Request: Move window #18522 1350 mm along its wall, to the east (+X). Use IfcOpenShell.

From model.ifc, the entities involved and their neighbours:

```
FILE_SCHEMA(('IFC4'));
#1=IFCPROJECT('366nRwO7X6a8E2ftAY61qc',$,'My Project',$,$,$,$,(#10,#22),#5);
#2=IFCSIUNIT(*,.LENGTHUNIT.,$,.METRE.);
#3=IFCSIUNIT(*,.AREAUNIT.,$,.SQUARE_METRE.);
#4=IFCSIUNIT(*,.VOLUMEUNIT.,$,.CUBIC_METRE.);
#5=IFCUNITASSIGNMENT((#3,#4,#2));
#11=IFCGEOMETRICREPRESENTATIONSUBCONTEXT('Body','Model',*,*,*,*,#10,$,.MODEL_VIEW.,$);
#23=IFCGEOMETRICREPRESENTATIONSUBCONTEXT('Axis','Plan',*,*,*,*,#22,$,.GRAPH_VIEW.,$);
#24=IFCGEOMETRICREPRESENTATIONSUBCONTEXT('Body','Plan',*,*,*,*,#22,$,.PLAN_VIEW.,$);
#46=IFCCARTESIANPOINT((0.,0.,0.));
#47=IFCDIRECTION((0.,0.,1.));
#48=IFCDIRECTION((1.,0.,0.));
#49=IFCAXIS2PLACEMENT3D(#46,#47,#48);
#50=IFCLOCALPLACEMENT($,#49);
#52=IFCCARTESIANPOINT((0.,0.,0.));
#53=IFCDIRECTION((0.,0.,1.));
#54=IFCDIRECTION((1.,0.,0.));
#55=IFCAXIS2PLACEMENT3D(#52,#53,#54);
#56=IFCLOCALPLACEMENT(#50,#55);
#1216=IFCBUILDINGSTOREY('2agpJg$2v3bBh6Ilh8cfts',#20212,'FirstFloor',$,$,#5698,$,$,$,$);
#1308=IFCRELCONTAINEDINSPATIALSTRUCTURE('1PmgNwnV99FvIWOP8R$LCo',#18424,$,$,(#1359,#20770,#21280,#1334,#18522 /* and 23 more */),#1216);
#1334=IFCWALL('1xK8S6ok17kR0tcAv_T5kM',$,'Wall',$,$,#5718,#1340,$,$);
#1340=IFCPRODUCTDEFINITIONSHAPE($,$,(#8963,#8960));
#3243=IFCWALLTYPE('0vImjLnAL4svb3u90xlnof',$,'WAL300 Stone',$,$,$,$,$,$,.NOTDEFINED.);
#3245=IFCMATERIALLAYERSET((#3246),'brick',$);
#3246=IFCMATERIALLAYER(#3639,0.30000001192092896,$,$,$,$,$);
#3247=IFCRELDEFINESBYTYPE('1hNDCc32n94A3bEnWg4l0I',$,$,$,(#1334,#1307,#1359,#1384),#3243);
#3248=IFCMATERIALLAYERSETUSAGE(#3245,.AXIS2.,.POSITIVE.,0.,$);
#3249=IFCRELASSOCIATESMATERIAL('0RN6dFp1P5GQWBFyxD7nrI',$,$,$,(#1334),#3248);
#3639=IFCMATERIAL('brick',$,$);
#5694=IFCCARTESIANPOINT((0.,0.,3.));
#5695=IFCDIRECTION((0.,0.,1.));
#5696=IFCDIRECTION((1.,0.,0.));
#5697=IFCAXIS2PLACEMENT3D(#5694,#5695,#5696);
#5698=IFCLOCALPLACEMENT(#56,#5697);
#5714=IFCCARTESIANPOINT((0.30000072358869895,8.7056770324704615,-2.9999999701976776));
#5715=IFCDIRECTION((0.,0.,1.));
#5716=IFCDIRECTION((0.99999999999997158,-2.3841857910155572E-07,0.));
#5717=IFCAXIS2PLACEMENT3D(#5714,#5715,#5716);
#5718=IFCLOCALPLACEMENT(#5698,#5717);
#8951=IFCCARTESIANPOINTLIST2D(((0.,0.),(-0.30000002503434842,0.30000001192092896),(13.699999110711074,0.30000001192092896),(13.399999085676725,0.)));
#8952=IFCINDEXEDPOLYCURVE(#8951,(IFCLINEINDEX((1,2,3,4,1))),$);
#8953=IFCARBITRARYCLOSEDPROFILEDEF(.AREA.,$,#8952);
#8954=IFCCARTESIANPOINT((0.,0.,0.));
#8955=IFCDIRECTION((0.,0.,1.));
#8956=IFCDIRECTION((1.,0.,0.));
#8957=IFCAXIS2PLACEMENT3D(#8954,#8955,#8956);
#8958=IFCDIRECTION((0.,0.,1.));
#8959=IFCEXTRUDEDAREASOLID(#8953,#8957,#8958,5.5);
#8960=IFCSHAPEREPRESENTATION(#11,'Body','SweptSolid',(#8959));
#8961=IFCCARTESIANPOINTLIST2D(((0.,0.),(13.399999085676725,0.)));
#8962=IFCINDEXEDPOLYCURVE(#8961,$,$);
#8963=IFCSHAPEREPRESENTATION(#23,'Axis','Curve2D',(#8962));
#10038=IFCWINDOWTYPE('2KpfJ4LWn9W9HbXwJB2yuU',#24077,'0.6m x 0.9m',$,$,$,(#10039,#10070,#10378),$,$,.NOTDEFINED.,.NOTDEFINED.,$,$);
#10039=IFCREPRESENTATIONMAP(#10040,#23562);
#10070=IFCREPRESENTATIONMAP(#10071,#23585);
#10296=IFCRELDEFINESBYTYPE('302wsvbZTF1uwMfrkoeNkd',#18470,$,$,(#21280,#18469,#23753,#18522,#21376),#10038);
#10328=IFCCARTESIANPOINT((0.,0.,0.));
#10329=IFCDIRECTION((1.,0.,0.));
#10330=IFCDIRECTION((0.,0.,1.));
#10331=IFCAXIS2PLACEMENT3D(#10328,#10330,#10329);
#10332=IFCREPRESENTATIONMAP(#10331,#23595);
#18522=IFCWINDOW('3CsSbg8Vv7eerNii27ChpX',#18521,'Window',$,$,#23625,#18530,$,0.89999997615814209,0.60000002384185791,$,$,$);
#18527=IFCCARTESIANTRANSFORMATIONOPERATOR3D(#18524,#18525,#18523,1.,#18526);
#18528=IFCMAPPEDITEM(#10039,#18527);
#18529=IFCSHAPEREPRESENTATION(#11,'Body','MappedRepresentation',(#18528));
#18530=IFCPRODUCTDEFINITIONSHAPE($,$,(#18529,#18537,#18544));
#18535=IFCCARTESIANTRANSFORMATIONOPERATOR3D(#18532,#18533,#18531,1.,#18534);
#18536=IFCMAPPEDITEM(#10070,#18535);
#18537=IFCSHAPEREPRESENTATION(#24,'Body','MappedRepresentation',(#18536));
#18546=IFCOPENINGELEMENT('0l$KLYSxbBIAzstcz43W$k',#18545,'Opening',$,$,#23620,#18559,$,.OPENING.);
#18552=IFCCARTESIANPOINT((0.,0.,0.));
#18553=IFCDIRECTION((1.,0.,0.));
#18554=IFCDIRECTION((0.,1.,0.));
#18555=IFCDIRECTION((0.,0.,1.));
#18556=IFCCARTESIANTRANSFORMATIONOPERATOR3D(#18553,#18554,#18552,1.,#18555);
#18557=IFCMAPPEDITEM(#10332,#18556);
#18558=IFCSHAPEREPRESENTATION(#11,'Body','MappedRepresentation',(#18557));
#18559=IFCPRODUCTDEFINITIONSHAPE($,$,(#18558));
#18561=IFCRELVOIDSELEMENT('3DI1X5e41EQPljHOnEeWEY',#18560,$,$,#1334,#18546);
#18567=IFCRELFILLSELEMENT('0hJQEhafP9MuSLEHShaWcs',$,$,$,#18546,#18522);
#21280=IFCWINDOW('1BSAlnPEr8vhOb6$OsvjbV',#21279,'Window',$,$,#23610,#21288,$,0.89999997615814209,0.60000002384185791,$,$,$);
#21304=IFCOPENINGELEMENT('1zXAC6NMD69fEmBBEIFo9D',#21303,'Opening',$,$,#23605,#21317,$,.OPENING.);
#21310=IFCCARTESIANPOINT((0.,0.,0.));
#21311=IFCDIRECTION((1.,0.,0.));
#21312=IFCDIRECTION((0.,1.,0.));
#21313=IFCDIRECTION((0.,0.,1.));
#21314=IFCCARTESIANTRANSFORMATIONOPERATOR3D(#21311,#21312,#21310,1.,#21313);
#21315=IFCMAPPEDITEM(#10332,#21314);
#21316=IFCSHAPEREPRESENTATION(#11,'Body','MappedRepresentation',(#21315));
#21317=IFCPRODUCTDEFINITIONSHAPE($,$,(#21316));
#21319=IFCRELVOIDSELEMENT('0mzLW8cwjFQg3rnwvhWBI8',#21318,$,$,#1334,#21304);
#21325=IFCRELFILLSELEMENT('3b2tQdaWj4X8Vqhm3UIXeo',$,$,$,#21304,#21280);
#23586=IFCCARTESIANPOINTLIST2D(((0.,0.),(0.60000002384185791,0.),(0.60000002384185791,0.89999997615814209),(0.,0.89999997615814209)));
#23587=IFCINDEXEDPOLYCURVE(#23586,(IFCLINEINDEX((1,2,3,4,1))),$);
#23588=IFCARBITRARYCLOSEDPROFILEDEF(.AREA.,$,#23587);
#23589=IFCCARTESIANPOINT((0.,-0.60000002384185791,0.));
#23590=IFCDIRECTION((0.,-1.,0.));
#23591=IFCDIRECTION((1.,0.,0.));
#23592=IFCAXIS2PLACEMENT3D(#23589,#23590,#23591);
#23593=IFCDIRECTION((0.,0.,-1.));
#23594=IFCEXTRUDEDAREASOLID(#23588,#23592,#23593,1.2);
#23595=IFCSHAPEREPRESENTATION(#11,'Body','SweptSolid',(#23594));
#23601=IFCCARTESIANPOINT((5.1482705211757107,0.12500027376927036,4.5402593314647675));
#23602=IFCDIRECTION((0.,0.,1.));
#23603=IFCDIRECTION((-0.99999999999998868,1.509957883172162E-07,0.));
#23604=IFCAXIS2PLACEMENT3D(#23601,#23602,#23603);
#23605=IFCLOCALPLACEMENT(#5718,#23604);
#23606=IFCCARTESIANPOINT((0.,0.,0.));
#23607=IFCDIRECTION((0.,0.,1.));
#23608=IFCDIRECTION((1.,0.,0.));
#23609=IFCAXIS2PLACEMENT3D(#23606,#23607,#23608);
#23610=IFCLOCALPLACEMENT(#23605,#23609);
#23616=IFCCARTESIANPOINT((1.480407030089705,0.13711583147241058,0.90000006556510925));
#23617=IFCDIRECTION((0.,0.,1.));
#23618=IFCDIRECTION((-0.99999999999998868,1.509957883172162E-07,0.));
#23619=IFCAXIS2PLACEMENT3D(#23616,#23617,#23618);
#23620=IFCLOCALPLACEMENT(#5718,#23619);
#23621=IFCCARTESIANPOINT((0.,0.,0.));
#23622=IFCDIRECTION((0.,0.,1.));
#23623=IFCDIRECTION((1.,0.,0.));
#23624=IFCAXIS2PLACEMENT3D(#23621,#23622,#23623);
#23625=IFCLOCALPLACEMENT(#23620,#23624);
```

```python
import ifcopenshell
import ifcopenshell.api.geometry
import ifcopenshell.util.placement

model = ifcopenshell.open("model.ifc")

window = model.by_id(18522)
opening = window.FillsVoids[0].RelatingOpeningElement
wall = opening.VoidsElements[0].RelatingBuildingElement

wall_matrix = ifcopenshell.util.placement.get_local_placement(wall.ObjectPlacement)
shift = wall_matrix[:3, 0] * 1.35
before = ifcopenshell.util.placement.get_local_placement(window.ObjectPlacement)[:3, 3].copy()

# The window is placed relative to its opening, so it follows when the opening moves.
matrix = ifcopenshell.util.placement.get_local_placement(opening.ObjectPlacement)
matrix[:3, 3] += shift
ifcopenshell.api.geometry.edit_object_placement(
    model, product=opening, matrix=matrix, is_si=False, should_transform_children=True
)

after = ifcopenshell.util.placement.get_local_placement(window.ObjectPlacement)[:3, 3]
print("window moved by", (after - before).round(3) + 0.0)

model.write("model_v2.ifc")
```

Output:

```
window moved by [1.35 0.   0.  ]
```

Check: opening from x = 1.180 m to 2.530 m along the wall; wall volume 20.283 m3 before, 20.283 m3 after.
